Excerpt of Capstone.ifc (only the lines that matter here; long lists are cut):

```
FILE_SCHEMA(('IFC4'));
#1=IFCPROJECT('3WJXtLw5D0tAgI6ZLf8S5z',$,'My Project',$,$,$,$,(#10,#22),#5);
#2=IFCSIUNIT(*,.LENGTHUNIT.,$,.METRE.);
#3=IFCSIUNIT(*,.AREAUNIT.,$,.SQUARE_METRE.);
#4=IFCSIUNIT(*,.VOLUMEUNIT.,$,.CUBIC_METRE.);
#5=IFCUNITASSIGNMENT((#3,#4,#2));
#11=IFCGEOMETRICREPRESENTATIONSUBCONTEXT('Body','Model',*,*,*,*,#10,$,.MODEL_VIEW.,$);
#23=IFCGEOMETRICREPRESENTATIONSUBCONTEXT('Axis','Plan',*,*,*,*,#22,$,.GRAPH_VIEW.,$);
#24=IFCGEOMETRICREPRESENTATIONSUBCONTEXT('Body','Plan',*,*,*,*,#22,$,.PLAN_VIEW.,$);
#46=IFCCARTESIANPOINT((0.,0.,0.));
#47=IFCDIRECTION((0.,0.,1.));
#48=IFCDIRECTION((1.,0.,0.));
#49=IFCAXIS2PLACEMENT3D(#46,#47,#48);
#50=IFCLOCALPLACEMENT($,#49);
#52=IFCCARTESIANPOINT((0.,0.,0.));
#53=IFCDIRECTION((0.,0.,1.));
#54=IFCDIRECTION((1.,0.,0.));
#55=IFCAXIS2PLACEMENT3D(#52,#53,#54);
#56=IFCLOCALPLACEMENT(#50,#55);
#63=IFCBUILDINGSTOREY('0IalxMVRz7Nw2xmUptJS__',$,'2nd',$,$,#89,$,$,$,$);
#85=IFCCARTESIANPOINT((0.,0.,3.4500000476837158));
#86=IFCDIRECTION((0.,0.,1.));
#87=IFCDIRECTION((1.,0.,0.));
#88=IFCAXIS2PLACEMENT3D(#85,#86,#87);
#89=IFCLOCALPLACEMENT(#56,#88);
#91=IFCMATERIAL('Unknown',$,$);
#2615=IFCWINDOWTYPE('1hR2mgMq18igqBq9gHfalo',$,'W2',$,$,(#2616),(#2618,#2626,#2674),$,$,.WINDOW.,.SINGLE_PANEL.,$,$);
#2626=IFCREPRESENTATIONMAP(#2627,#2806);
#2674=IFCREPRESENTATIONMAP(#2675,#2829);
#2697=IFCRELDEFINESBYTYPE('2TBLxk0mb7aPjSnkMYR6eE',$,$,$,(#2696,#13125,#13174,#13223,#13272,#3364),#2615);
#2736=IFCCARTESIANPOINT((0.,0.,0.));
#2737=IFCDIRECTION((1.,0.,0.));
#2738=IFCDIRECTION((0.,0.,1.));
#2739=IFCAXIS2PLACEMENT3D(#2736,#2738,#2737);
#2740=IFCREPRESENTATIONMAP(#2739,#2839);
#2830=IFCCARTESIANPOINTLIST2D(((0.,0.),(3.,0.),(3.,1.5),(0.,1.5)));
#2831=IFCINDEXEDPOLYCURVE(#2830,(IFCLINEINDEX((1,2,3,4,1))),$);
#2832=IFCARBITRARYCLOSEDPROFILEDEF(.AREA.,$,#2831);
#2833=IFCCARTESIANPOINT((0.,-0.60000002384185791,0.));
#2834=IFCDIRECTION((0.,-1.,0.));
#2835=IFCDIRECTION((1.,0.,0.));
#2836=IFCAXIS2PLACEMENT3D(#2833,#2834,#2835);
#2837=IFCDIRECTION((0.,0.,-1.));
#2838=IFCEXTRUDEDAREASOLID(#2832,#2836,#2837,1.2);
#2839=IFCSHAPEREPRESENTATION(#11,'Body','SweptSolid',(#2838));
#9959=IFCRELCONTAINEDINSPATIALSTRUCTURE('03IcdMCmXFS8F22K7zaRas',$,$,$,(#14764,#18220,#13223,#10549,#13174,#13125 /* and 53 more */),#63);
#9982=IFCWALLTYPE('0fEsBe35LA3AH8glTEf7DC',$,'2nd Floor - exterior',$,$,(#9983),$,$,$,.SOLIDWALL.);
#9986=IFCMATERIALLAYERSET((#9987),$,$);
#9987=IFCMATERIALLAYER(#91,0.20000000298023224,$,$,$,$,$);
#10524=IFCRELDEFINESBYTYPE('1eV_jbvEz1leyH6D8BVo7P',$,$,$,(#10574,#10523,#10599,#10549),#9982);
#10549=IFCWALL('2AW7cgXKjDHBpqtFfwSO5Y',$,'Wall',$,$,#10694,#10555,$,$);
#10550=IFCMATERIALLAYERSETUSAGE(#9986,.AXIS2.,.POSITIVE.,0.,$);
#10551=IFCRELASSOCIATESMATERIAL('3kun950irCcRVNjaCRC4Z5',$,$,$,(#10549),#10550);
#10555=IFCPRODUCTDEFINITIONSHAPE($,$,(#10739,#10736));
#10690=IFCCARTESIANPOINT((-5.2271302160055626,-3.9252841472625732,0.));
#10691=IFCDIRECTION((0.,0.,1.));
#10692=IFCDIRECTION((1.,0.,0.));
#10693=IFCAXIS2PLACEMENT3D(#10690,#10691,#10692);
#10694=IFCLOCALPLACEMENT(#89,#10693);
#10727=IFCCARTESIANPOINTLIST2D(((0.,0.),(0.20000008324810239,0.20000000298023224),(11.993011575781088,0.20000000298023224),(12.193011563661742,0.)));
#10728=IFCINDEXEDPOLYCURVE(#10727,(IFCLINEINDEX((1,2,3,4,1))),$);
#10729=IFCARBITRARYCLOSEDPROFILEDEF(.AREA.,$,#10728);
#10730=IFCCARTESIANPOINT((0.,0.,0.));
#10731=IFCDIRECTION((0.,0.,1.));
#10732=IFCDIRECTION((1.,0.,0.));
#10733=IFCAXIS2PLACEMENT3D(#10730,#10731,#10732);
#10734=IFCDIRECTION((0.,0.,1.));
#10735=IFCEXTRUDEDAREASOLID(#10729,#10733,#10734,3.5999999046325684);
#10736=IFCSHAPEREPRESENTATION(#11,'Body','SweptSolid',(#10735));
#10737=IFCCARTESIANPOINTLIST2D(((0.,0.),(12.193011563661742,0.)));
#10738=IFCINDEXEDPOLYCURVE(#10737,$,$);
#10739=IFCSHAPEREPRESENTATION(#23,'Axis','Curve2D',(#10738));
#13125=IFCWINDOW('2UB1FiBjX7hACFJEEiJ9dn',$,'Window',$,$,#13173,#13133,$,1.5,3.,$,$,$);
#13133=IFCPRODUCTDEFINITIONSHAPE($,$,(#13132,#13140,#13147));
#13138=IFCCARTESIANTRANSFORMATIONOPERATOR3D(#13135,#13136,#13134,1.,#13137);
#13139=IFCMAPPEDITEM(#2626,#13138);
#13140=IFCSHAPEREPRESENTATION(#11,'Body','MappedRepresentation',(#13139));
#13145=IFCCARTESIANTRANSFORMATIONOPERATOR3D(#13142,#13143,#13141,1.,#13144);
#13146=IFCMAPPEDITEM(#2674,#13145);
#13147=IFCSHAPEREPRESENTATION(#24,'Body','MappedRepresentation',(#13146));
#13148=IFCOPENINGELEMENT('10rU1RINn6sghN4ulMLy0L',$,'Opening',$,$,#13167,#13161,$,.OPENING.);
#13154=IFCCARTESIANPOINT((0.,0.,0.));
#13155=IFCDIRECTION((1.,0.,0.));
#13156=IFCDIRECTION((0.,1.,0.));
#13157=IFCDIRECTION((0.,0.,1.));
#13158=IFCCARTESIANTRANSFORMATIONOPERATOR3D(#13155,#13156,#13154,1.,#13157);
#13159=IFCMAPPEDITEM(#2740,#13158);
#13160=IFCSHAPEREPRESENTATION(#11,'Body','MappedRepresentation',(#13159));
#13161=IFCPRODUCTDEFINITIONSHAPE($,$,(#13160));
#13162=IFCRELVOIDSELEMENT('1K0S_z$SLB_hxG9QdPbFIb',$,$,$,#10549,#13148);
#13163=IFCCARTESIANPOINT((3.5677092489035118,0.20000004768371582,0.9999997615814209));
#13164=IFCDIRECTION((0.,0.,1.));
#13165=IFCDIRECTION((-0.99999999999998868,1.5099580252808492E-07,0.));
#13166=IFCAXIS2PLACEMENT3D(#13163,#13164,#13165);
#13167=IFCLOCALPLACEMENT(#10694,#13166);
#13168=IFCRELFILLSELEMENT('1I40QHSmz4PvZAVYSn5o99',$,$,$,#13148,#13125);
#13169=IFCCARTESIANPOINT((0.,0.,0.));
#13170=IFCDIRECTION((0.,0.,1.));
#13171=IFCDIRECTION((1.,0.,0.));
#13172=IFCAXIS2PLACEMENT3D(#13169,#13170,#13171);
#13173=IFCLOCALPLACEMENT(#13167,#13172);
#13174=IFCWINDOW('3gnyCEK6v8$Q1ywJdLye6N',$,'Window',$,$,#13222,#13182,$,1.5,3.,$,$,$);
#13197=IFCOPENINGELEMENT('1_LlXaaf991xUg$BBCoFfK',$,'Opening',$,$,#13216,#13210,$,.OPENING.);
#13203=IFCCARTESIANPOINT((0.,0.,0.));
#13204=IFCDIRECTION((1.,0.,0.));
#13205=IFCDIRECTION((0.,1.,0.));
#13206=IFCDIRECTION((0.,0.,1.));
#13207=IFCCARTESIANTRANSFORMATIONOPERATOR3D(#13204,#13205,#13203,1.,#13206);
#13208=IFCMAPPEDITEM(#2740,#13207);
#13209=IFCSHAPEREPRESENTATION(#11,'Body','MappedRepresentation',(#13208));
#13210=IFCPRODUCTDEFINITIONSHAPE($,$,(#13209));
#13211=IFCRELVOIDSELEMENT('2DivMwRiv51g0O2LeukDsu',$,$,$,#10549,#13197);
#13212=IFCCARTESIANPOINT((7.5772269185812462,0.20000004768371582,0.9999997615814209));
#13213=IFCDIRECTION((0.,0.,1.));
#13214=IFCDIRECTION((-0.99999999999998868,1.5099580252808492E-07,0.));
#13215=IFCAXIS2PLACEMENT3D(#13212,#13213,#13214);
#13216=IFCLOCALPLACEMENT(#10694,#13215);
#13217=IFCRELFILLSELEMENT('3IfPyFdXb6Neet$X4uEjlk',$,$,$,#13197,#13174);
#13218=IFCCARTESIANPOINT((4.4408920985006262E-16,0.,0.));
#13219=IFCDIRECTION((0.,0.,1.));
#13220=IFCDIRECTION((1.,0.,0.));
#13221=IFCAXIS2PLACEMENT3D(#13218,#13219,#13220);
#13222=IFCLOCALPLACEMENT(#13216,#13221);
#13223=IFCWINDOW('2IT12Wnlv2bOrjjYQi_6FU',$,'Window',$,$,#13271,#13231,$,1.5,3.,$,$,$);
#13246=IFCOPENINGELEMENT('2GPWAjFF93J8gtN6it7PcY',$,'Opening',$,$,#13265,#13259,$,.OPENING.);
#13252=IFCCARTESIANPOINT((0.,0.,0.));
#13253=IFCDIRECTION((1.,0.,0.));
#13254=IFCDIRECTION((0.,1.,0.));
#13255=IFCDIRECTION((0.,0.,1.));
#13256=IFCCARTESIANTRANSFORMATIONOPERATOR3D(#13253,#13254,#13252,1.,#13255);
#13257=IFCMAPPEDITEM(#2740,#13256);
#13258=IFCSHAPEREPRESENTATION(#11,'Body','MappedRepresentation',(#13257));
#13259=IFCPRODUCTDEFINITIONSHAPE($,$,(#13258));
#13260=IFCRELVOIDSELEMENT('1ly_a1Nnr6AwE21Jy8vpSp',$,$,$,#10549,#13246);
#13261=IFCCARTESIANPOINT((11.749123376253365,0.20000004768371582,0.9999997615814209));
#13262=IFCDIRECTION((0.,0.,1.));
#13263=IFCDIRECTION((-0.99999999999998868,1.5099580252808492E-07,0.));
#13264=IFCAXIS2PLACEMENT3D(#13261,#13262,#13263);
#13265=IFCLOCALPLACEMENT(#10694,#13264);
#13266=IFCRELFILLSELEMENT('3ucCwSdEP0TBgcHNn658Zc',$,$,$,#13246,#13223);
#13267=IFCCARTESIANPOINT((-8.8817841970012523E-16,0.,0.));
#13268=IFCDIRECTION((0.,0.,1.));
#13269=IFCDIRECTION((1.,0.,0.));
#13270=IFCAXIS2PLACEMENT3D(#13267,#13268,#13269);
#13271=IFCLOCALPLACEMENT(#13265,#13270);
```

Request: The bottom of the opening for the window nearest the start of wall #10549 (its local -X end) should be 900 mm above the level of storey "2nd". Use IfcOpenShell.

```python
import numpy as np
import ifcopenshell
import ifcopenshell.api.geometry
import ifcopenshell.geom
import ifcopenshell.util.element
import ifcopenshell.util.placement
import ifcopenshell.util.shape
import ifcopenshell.util.unit

model = ifcopenshell.open("Capstone.ifc")
unit_scale = ifcopenshell.util.unit.calculate_unit_scale(model)

window = model.by_guid("2UB1FiBjX7hACFJEEiJ9dn")
opening = window.FillsVoids[0].RelatingOpeningElement
storey = ifcopenshell.util.element.get_container(window, ifc_class="IfcBuildingStorey")
level = ifcopenshell.util.placement.get_local_placement(storey.ObjectPlacement)[2, 3]

# The opening's origin need not be at the sill, so measure its lowest point.
shape = ifcopenshell.geom.create_shape(ifcopenshell.geom.settings(), opening)
bottom = ifcopenshell.util.shape.get_shape_bottom_elevation(shape, shape.geometry) / unit_scale
dz = level + 0.9 - bottom

shift = np.array([0.0, 0.0, dz])
# The window is placed relative to its opening, so it follows when the opening moves.
matrix = ifcopenshell.util.placement.get_local_placement(opening.ObjectPlacement)
matrix[:3, 3] += shift
ifcopenshell.api.geometry.edit_object_placement(
    model, product=opening, matrix=matrix, is_si=False, should_transform_children=True
)

print(f"moved by {dz * unit_scale:+.3f} m")

model.write("Capstone_v2.ifc")
```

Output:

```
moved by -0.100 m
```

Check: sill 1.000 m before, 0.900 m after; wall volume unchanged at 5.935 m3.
